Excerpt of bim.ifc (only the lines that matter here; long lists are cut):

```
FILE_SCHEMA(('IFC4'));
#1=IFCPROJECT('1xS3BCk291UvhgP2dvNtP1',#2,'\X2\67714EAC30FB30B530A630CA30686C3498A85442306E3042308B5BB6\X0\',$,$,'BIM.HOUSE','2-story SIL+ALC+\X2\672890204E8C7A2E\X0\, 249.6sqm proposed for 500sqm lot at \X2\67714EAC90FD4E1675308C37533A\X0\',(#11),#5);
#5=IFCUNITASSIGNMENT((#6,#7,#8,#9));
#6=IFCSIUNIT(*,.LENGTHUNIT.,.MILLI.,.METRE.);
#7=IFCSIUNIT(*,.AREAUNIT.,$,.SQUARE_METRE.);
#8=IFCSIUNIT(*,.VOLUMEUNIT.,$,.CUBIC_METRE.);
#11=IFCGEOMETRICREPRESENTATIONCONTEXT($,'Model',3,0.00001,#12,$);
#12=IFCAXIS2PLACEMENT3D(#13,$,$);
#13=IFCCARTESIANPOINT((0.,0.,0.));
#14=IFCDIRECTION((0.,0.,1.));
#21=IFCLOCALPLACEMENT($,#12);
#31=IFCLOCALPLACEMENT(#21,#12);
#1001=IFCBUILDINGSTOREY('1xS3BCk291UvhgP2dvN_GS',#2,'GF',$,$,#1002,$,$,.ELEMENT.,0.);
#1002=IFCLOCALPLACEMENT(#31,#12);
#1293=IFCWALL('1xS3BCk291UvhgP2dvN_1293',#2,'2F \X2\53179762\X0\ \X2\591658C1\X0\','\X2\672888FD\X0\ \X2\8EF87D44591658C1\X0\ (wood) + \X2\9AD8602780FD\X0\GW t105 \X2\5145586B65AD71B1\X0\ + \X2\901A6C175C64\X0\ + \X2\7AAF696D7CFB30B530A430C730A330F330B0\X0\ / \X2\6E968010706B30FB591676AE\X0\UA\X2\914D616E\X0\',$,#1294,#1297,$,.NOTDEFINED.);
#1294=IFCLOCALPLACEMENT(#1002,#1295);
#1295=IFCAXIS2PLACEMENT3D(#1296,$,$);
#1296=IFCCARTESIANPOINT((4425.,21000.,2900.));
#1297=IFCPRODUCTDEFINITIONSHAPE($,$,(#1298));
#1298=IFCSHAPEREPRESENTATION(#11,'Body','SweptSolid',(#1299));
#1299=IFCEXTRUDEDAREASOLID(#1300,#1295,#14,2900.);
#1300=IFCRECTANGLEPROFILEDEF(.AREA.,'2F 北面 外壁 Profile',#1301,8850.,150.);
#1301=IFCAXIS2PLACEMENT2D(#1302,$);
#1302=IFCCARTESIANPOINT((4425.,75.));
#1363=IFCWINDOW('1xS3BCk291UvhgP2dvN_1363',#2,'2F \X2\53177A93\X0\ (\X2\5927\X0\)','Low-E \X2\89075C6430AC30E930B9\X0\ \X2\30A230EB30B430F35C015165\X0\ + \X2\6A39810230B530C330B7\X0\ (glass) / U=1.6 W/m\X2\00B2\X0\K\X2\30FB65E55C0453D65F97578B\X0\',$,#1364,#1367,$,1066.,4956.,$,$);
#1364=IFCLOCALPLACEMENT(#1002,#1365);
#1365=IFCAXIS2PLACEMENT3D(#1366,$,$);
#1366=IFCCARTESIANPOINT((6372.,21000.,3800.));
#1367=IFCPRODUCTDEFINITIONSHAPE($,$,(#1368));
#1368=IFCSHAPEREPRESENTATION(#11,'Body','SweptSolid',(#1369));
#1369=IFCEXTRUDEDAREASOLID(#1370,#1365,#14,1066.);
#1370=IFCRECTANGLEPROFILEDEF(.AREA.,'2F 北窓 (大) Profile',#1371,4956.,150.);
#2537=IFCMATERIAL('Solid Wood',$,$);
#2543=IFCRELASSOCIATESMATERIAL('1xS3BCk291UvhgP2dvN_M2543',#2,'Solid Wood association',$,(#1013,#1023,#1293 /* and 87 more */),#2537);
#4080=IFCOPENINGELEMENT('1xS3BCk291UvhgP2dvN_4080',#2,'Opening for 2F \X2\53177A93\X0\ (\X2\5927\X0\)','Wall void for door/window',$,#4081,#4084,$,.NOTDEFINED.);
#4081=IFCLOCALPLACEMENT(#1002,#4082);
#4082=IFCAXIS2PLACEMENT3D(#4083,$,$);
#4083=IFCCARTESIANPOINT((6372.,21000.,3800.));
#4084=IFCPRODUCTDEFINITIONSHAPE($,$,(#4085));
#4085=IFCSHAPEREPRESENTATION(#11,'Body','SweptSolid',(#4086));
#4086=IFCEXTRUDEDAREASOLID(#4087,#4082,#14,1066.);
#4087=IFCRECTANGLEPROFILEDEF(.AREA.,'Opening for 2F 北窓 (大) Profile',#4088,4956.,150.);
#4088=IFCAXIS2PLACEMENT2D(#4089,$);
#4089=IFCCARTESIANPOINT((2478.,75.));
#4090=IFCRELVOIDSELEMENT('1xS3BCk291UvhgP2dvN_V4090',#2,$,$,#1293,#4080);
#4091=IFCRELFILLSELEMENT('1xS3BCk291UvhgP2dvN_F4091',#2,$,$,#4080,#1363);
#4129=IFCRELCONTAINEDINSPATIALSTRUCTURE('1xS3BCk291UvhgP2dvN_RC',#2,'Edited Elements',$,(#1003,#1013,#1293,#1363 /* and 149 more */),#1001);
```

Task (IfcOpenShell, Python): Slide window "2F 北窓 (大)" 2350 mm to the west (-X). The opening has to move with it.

```python
import ifcopenshell
import ifcopenshell.api.geometry
import ifcopenshell.util.placement

model = ifcopenshell.open("bim.ifc")

window = model.by_guid("1xS3BCk291UvhgP2dvN_1363")
opening = window.FillsVoids[0].RelatingOpeningElement
wall = opening.VoidsElements[0].RelatingBuildingElement

wall_matrix = ifcopenshell.util.placement.get_local_placement(wall.ObjectPlacement)
shift = wall_matrix[:3, 0] * -2350.0
before = ifcopenshell.util.placement.get_local_placement(window.ObjectPlacement)[:3, 3].copy()

# The window is not placed relative to its opening, so move both.
for product in (opening, window):
    matrix = ifcopenshell.util.placement.get_local_placement(product.ObjectPlacement)
    matrix[:3, 3] += shift
    ifcopenshell.api.geometry.edit_object_placement(model, product=product, matrix=matrix, is_si=False)

after = ifcopenshell.util.placement.get_local_placement(window.ObjectPlacement)[:3, 3]
print("window moved by", (after - before).round(3) + 0.0)

model.write("bim_edited.ifc")
```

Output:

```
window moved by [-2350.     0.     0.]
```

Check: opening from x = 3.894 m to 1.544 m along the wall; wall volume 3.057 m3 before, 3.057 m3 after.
